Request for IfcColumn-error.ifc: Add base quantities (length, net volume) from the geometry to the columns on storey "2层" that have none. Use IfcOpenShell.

First a look at what the model holds.

```python
import ifcopenshell
import ifcopenshell.util.element
import ifcopenshell.util.unit

model = ifcopenshell.open("IfcColumn-error.ifc")
print(model.schema)
for unit_type in ("LENGTHUNIT", "AREAUNIT", "VOLUMEUNIT"):
    print(unit_type, ifcopenshell.util.unit.calculate_unit_scale(model, unit_type))
storey = next(s for s in model.by_type("IfcBuildingStorey") if s.Name == "2层")
columns = [e for e in ifcopenshell.util.element.get_decomposition(storey) if e.is_a("IfcColumn")]
for e in sorted(columns, key=lambda e: e.id()):
    print(e.id(), e.is_a(), e.Name, list(ifcopenshell.util.element.get_psets(e, qtos_only=True)), sep=" | ")
```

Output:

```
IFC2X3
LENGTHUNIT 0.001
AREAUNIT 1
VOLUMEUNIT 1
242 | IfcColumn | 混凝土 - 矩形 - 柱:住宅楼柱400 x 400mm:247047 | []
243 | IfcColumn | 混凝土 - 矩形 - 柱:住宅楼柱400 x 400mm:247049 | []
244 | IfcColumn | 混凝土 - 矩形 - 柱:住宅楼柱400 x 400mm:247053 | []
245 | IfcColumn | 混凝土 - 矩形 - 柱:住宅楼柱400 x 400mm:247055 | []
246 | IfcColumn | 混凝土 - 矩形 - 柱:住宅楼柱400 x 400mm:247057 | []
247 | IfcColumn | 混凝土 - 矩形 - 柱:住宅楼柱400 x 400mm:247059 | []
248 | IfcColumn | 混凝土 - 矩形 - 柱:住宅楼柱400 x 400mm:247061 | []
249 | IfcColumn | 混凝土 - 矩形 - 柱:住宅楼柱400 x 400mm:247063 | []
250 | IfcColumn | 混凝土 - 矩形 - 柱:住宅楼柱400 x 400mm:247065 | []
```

```python
import ifcopenshell
import ifcopenshell.api.pset
import ifcopenshell.geom
import ifcopenshell.util.element
import ifcopenshell.util.shape
import ifcopenshell.util.unit

model = ifcopenshell.open("IfcColumn-error.ifc")
unit_scale = ifcopenshell.util.unit.calculate_unit_scale(model)
volume_scale = ifcopenshell.util.unit.calculate_unit_scale(model, "VOLUMEUNIT")
settings = ifcopenshell.geom.settings()

storey = next(s for s in model.by_type("IfcBuildingStorey") if s.Name == "2层")
columns = [e for e in ifcopenshell.util.element.get_decomposition(storey) if e.is_a("IfcColumn")]

for e in sorted(columns, key=lambda e: e.id()):
    if ifcopenshell.util.element.get_psets(e, qtos_only=True, should_inherit=False):
        continue
    # Geometry comes back in metres, in the element's own axes.
    shape = ifcopenshell.geom.create_shape(settings, e)
    values = {
        "Length": ifcopenshell.util.shape.get_z(shape.geometry) / unit_scale,
        "NetVolume": ifcopenshell.util.shape.get_volume(shape.geometry) / volume_scale,
    }
    qto = ifcopenshell.api.pset.add_qto(model, product=e, name="BaseQuantities")
    ifcopenshell.api.pset.edit_qto(model, qto=qto, properties=values)
    print(e.id(), {k: round(v, 3) for k, v in values.items()})

model.write("IfcColumn-error_v2.ifc")
```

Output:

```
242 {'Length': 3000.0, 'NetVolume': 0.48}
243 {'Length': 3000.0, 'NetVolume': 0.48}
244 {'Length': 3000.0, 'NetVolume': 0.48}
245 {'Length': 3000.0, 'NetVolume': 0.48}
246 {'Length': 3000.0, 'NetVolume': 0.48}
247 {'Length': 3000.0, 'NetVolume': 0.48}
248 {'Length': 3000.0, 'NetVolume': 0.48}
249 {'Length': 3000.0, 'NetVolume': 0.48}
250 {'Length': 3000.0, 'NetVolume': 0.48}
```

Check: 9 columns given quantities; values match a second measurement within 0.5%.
